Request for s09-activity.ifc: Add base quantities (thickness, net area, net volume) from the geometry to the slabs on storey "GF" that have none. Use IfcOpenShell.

First a look at what the model holds.

```python
import ifcopenshell
import ifcopenshell.util.element
import ifcopenshell.util.unit

model = ifcopenshell.open("s09-activity.ifc")
print(model.schema)
for unit_type in ("LENGTHUNIT", "AREAUNIT", "VOLUMEUNIT"):
    print(unit_type, ifcopenshell.util.unit.calculate_unit_scale(model, unit_type))
storey = next(s for s in model.by_type("IfcBuildingStorey") if s.Name == "GF")
slabs = [e for e in ifcopenshell.util.element.get_decomposition(storey) if e.is_a("IfcSlab")]
for e in sorted(slabs, key=lambda e: e.id()):
    print(e.id(), e.is_a(), e.Name, list(ifcopenshell.util.element.get_psets(e, qtos_only=True)), sep=" | ")
```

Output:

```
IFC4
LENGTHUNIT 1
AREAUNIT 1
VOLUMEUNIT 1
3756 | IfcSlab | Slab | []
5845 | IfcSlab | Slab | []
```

```python
import ifcopenshell
import ifcopenshell.api.pset
import ifcopenshell.geom
import ifcopenshell.util.element
import ifcopenshell.util.shape
import ifcopenshell.util.unit

model = ifcopenshell.open("s09-activity.ifc")
unit_scale = ifcopenshell.util.unit.calculate_unit_scale(model)
area_scale = ifcopenshell.util.unit.calculate_unit_scale(model, "AREAUNIT")
volume_scale = ifcopenshell.util.unit.calculate_unit_scale(model, "VOLUMEUNIT")
settings = ifcopenshell.geom.settings()

storey = next(s for s in model.by_type("IfcBuildingStorey") if s.Name == "GF")
slabs = [e for e in ifcopenshell.util.element.get_decomposition(storey) if e.is_a("IfcSlab")]

for e in sorted(slabs, key=lambda e: e.id()):
    if ifcopenshell.util.element.get_psets(e, qtos_only=True, should_inherit=False):
        continue
    # Geometry comes back in metres, in the element's own axes.
    shape = ifcopenshell.geom.create_shape(settings, e)
    values = {
        "Width": ifcopenshell.util.shape.get_z(shape.geometry) / unit_scale,
        "NetArea": ifcopenshell.util.shape.get_footprint_area(shape.geometry) / area_scale,
        "NetVolume": ifcopenshell.util.shape.get_volume(shape.geometry) / volume_scale,
    }
    qto = ifcopenshell.api.pset.add_qto(model, product=e, name="Qto_SlabBaseQuantities")
    ifcopenshell.api.pset.edit_qto(model, qto=qto, properties=values)
    print(e.id(), {k: round(v, 3) for k, v in values.items()})

model.write("s09-activity_edited.ifc")
```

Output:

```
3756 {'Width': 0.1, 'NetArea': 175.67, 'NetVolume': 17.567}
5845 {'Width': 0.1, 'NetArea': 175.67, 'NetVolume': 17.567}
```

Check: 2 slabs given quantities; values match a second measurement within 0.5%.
